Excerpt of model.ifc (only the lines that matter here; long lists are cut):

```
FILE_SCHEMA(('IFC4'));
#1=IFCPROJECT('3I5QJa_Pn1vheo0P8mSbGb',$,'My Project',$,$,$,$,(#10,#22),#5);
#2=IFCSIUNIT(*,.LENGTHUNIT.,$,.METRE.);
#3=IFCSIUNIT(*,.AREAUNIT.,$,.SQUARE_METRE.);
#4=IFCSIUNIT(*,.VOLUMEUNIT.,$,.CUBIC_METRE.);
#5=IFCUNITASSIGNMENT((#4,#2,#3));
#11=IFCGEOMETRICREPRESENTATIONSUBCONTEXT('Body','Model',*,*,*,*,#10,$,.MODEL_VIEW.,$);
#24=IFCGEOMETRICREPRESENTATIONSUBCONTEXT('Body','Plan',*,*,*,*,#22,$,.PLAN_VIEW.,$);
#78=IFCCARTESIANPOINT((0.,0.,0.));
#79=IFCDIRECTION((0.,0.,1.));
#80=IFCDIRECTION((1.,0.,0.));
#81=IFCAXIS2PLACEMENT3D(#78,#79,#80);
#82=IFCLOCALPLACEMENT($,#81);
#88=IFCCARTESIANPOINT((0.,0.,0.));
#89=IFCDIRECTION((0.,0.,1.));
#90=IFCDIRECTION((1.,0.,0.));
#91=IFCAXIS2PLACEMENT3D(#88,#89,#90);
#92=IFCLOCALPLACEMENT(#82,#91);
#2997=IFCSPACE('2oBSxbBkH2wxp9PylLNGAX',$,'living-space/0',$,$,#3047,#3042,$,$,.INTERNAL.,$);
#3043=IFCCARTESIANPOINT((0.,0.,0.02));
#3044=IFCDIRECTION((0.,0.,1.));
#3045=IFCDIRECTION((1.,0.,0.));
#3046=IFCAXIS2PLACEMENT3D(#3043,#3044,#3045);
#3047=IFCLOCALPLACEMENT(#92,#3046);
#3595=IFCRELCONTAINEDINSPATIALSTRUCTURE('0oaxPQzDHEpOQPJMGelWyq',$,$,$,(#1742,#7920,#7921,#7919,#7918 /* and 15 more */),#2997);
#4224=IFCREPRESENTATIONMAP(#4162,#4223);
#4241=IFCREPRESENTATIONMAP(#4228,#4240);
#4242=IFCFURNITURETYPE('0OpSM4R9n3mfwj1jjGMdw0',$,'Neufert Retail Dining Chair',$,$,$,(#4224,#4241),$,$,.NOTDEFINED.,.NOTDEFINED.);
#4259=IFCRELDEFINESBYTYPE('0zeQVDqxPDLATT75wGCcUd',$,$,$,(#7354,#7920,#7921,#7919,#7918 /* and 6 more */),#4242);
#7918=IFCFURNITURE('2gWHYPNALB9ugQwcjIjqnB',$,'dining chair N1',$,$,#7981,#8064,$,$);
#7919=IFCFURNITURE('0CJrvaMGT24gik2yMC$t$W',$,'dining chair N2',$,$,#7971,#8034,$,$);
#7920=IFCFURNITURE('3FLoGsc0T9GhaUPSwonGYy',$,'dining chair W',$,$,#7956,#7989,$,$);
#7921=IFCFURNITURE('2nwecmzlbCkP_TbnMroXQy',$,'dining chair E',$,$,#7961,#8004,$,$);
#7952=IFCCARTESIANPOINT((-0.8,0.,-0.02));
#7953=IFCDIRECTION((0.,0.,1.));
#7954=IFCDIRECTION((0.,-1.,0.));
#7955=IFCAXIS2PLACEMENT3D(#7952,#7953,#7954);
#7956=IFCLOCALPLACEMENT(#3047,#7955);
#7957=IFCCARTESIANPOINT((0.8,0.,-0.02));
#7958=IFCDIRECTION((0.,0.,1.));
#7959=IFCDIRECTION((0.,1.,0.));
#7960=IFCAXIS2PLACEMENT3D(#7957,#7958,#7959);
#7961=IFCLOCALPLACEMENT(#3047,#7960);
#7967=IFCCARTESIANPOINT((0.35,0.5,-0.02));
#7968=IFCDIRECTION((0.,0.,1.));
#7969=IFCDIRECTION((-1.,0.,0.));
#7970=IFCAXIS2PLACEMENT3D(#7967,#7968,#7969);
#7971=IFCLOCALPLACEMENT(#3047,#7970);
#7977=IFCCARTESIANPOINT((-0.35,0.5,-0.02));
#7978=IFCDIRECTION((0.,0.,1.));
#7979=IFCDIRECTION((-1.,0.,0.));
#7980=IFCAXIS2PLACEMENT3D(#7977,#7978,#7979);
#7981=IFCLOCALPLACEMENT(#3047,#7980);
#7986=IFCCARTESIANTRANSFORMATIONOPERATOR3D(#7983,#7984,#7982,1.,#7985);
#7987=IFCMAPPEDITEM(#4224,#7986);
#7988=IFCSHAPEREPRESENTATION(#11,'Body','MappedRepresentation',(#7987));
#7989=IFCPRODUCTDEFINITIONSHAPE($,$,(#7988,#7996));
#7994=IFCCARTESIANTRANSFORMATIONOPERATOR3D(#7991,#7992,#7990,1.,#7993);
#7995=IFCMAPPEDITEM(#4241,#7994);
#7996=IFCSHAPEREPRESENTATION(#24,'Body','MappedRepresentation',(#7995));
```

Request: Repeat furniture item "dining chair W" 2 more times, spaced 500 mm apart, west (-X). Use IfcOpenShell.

```python
import numpy as np
import ifcopenshell
import ifcopenshell.api.geometry
import ifcopenshell.api.root
import ifcopenshell.util.element
import ifcopenshell.util.placement

model = ifcopenshell.open("model.ifc")

source = model.by_guid("3FLoGsc0T9GhaUPSwonGYy")
base = ifcopenshell.util.placement.get_local_placement(source.ObjectPlacement)
step = np.array([-1.0, 0.0, 0.0]) * 0.5

for i in range(1, 3):
    copy = ifcopenshell.api.root.copy_class(model, product=source)
    copy.Representation = ifcopenshell.util.element.copy_deep(
        model, source.Representation, exclude=["IfcGeometricRepresentationContext", "IfcRepresentationMap"]
    )
    matrix = base.copy()
    matrix[:3, 3] += i * step
    print("added at", matrix[:3, 3].round(3) + 0.0)
    ifcopenshell.api.geometry.edit_object_placement(model, product=copy, matrix=matrix, is_si=False)

model.write("model_edited.ifc")
```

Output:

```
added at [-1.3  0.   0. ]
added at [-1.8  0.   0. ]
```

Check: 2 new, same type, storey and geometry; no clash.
